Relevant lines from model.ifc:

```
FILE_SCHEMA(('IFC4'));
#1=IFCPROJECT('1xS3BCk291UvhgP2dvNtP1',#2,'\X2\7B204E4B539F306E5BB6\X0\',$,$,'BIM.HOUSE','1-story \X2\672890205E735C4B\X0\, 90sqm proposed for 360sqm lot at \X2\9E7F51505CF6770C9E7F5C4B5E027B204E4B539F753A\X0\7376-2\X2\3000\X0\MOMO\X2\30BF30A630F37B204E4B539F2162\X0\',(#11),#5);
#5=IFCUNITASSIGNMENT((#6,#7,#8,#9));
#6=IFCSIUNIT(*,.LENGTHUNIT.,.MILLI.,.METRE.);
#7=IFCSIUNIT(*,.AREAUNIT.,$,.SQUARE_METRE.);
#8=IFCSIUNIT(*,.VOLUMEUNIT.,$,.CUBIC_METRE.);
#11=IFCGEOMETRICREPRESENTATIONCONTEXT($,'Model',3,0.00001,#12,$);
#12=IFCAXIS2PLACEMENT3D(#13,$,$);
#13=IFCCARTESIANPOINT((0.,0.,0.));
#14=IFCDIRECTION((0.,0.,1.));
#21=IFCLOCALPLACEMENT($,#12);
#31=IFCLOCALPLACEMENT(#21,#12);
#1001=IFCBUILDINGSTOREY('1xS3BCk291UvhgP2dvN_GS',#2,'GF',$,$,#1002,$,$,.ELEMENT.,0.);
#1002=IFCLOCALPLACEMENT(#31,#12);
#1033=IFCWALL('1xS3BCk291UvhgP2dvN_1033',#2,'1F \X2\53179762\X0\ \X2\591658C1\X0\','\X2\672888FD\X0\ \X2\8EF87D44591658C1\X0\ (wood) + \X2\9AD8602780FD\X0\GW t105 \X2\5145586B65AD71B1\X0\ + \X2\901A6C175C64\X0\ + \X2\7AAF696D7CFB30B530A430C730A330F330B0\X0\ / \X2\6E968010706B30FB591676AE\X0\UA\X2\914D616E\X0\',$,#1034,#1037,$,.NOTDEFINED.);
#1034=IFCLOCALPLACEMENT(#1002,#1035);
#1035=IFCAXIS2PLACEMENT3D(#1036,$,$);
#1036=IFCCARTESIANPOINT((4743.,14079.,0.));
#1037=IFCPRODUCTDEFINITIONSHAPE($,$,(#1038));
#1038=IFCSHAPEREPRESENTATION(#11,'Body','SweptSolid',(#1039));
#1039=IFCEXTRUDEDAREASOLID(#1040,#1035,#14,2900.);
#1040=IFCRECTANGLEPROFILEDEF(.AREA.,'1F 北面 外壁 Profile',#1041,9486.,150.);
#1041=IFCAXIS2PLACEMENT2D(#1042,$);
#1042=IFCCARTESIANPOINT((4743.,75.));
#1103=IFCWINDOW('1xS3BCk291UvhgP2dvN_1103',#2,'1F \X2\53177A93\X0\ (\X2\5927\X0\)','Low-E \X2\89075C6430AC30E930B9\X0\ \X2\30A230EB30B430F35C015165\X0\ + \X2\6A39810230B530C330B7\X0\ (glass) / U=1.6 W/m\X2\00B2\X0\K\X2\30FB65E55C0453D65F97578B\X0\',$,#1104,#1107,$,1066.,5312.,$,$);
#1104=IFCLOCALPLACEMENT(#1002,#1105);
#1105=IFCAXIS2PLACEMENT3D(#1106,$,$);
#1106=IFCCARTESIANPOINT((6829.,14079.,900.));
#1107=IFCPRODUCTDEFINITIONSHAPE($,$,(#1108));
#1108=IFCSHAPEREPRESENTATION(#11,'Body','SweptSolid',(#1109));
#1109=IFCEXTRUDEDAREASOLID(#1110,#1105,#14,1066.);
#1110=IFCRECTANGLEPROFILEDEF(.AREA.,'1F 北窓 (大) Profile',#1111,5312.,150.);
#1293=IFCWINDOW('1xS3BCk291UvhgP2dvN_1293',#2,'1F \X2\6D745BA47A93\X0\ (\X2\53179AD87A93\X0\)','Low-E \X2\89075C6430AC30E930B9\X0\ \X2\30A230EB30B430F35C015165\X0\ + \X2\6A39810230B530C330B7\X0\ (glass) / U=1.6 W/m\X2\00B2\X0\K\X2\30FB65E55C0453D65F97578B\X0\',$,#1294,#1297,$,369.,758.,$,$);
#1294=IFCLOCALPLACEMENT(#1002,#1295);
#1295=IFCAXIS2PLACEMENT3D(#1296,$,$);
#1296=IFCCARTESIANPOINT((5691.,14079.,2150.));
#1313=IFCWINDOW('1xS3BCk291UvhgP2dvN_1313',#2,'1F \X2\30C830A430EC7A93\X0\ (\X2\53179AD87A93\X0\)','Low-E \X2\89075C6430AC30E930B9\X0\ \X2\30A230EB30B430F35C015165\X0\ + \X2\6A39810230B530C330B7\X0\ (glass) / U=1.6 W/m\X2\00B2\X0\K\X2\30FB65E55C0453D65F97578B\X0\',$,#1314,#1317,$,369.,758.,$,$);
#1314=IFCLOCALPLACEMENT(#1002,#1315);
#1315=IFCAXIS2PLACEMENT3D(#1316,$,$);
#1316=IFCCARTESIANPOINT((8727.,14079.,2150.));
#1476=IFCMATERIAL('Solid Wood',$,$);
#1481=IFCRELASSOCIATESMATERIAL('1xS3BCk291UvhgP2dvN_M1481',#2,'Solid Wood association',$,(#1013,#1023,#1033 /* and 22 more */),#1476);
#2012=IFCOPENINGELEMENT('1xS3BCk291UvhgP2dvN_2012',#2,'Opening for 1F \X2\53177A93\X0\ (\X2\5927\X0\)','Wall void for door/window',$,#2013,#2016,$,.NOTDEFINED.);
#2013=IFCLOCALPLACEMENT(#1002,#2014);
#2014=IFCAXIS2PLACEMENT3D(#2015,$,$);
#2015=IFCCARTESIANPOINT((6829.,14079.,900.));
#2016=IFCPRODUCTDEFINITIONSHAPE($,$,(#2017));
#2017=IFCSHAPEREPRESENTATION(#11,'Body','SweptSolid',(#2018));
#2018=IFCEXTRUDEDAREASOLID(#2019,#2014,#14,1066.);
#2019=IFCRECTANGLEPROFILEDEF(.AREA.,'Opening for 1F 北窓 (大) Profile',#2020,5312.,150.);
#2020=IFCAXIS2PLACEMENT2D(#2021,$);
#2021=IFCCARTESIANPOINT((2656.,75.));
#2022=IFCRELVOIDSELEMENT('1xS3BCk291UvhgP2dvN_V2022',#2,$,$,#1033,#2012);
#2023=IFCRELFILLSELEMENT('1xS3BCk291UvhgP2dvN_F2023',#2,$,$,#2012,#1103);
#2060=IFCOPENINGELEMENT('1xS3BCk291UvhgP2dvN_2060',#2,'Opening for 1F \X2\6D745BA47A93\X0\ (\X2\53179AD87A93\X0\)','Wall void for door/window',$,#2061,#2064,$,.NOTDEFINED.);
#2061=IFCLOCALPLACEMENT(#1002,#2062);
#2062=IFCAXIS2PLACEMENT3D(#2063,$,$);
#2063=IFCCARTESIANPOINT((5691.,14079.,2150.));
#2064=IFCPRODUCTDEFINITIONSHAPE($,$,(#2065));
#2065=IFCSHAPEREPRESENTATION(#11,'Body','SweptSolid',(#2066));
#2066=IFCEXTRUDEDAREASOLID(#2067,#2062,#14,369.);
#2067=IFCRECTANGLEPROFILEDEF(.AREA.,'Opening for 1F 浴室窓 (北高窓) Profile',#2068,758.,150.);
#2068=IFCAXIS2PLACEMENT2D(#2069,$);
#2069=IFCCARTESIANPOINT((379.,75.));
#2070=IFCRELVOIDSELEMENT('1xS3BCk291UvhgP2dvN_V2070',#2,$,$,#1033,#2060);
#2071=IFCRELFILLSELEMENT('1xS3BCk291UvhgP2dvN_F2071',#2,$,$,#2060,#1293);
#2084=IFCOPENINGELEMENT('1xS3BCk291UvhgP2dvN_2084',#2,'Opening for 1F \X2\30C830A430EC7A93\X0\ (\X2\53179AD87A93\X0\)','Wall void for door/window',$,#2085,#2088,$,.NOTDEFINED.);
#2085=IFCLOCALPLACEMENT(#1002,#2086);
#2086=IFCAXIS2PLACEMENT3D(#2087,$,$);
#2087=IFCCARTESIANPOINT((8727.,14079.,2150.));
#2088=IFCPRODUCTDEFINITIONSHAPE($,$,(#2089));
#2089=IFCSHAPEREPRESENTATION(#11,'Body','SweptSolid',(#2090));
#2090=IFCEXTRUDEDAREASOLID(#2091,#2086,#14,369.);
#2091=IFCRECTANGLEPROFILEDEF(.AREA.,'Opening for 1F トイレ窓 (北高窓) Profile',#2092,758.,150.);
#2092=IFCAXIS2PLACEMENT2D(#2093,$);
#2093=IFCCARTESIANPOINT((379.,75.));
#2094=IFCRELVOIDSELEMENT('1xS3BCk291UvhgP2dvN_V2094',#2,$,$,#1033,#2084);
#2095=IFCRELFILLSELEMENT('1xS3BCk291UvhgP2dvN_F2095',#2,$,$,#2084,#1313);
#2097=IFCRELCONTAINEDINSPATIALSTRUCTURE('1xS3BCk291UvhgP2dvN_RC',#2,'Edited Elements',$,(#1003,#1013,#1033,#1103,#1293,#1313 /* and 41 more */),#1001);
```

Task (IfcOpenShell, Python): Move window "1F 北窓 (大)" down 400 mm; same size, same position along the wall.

```python
import numpy as np
import ifcopenshell
import ifcopenshell.api.geometry
import ifcopenshell.util.placement
import ifcopenshell.util.unit

model = ifcopenshell.open("model.ifc")
unit_scale = ifcopenshell.util.unit.calculate_unit_scale(model)

window = model.by_id(1103)
opening = window.FillsVoids[0].RelatingOpeningElement
dz = -400.0

shift = np.array([0.0, 0.0, dz])
# The window is not placed relative to its opening, so move both.
for product in (opening, window):
    matrix = ifcopenshell.util.placement.get_local_placement(product.ObjectPlacement)
    matrix[:3, 3] += shift
    ifcopenshell.api.geometry.edit_object_placement(model, product=product, matrix=matrix, is_si=False)

print(f"moved by {dz * unit_scale:+.3f} m")

model.write("model-out.ifc")
```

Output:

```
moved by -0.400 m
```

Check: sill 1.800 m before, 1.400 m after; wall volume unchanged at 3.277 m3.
